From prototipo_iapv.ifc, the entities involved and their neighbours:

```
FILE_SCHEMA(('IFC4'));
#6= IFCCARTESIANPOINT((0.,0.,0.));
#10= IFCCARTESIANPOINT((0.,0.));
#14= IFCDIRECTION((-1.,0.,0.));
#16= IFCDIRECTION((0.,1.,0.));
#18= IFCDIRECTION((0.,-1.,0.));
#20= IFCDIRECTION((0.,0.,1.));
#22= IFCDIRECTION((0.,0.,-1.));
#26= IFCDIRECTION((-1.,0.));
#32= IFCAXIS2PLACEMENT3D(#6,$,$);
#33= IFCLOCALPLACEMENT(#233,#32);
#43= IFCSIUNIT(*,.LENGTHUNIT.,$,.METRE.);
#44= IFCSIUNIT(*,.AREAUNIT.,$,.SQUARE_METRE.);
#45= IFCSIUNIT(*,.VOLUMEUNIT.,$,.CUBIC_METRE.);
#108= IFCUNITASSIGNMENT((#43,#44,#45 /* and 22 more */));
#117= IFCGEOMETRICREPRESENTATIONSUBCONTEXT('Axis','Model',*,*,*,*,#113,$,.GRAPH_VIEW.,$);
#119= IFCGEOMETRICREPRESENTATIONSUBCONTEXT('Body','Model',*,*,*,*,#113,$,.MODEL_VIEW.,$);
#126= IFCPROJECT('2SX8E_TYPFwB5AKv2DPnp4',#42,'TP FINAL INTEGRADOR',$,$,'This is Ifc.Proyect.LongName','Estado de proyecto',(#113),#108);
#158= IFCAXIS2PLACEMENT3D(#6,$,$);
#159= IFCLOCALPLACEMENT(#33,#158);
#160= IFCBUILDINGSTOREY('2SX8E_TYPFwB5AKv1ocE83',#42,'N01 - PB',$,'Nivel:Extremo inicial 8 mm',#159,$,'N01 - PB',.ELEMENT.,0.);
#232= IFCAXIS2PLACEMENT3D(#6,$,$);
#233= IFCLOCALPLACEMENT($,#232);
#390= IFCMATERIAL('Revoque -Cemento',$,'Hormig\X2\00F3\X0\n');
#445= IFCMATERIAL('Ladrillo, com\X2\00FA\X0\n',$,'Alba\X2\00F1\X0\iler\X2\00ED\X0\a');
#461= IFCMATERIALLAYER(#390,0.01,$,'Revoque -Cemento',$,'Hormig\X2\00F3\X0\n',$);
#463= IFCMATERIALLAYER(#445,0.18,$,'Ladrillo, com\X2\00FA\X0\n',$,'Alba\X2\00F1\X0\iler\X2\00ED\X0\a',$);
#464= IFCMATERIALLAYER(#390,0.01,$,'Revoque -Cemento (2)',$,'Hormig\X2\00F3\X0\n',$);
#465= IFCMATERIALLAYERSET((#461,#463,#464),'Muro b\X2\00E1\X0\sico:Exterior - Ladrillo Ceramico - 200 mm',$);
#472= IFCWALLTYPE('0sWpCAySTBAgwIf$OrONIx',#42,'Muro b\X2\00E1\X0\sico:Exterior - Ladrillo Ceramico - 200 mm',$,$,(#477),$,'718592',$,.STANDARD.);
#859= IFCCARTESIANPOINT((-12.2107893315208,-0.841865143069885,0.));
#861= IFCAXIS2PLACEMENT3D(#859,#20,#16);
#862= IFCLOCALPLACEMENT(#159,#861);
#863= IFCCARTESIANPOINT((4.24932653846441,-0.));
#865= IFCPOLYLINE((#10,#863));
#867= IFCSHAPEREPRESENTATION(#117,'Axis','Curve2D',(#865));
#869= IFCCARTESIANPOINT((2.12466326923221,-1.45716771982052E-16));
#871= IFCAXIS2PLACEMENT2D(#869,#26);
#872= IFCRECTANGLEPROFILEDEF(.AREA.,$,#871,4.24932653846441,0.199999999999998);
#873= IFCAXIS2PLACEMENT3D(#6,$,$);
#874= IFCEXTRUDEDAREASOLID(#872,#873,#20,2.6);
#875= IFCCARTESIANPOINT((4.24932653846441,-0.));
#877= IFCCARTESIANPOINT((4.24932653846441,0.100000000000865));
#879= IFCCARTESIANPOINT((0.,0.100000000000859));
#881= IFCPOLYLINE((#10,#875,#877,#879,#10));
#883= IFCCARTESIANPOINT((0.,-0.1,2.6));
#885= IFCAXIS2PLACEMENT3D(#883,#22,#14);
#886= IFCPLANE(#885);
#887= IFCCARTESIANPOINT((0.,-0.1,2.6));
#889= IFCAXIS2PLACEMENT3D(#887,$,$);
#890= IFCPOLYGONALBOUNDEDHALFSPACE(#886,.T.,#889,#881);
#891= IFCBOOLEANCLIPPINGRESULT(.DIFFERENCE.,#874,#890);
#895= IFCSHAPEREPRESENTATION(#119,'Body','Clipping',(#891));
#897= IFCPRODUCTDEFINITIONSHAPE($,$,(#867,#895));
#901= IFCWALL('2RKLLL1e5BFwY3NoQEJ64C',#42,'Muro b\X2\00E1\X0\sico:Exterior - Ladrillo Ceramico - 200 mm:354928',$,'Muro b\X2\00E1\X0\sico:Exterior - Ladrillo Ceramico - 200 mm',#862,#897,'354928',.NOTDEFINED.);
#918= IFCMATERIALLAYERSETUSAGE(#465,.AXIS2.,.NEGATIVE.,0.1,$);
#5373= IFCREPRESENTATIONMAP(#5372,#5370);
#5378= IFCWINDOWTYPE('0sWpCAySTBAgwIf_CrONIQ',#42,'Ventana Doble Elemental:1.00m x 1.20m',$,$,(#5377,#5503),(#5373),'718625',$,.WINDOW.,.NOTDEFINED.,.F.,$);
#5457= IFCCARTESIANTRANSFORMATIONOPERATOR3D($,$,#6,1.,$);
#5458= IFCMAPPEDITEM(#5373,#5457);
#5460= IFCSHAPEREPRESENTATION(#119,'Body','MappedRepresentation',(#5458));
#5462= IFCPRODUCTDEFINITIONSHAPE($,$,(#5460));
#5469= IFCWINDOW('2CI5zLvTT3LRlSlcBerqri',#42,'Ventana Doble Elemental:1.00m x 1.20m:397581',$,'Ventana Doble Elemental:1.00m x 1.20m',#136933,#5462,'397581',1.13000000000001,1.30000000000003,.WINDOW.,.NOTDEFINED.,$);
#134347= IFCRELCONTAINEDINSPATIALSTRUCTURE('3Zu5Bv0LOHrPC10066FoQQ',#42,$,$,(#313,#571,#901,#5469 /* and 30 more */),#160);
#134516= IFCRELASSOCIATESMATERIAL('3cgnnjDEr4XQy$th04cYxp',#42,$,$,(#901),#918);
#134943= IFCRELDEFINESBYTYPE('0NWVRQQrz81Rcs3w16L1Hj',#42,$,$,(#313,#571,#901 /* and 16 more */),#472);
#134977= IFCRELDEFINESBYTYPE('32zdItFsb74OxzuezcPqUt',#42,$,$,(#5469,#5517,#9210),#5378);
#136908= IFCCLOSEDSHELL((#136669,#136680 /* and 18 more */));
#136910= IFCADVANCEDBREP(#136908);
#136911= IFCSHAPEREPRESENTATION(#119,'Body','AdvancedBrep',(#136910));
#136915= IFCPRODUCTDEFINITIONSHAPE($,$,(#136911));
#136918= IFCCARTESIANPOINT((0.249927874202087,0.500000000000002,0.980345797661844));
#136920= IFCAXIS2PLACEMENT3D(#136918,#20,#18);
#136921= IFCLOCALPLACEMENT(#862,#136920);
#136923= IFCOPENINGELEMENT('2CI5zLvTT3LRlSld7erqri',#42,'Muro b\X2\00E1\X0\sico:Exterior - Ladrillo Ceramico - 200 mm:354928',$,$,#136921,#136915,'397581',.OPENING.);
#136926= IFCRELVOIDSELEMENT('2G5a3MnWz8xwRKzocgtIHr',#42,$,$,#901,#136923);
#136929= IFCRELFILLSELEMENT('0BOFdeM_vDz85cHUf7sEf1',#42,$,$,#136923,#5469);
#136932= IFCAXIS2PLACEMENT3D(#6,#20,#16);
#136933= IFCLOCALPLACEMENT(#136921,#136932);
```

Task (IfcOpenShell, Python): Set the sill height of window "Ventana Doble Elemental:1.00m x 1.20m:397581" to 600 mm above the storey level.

```python
import numpy as np
import ifcopenshell
import ifcopenshell.api.geometry
import ifcopenshell.geom
import ifcopenshell.util.element
import ifcopenshell.util.placement
import ifcopenshell.util.shape
import ifcopenshell.util.unit

model = ifcopenshell.open("prototipo_iapv.ifc")
unit_scale = ifcopenshell.util.unit.calculate_unit_scale(model)

window = model.by_guid("2CI5zLvTT3LRlSlcBerqri")
opening = window.FillsVoids[0].RelatingOpeningElement
storey = ifcopenshell.util.element.get_container(window, ifc_class="IfcBuildingStorey")
level = ifcopenshell.util.placement.get_local_placement(storey.ObjectPlacement)[2, 3]

# The opening's origin need not be at the sill, so measure its lowest point.
shape = ifcopenshell.geom.create_shape(ifcopenshell.geom.settings(), opening)
bottom = ifcopenshell.util.shape.get_shape_bottom_elevation(shape, shape.geometry) / unit_scale
dz = level + 0.6 / unit_scale - bottom

shift = np.array([0.0, 0.0, dz])
# The window is placed relative to its opening, so it follows when the opening moves.
matrix = ifcopenshell.util.placement.get_local_placement(opening.ObjectPlacement)
matrix[:3, 3] += shift
ifcopenshell.api.geometry.edit_object_placement(
    model, product=opening, matrix=matrix, is_si=False, should_transform_children=True
)

print(f"moved by {dz * unit_scale:+.3f} m")

model.write("prototipo_iapv-out.ifc")
```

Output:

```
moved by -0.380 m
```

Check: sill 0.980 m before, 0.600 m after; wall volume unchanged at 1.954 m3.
